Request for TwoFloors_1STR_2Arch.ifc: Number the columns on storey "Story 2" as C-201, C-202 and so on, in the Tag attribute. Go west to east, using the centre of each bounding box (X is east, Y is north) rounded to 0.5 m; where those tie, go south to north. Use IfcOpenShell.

First a look at what the model holds.

```python
import ifcopenshell
import ifcopenshell.util.element
import ifcopenshell.util.placement

model = ifcopenshell.open("TwoFloors_1STR_2Arch.ifc")
print(model.schema)
storey = next(s for s in model.by_type("IfcBuildingStorey") if s.Name == "Story 2")
columns = [e for e in ifcopenshell.util.element.get_decomposition(storey) if e.is_a("IfcColumn")]
for e in sorted(columns, key=lambda e: e.id()):
    origin = ifcopenshell.util.placement.get_local_placement(e.ObjectPlacement)[:3, 3]
    print(e.id(), e.Tag, e.Name, origin.round(2) + 0.0, sep=" | ")
```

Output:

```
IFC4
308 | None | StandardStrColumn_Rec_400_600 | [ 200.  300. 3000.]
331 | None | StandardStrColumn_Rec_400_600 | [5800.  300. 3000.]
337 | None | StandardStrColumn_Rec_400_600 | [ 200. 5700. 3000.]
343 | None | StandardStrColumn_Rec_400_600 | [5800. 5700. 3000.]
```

```python
import ifcopenshell
import ifcopenshell.geom
import ifcopenshell.util.element
import ifcopenshell.util.shape

model = ifcopenshell.open("TwoFloors_1STR_2Arch.ifc")
settings = ifcopenshell.geom.settings()
settings.set("use-world-coords", True)


def centre(element):
    shape = ifcopenshell.geom.create_shape(settings, element)
    return ifcopenshell.util.shape.get_bbox_centroid(shape.geometry)


storey = next(s for s in model.by_type("IfcBuildingStorey") if s.Name == "Story 2")
columns = [e for e in ifcopenshell.util.element.get_decomposition(storey) if e.is_a("IfcColumn")]

# Insertion points can sit at a corner or the storey origin, so sort by the geometry (in metres).
centres = {e: centre(e) for e in columns}
columns.sort(key=lambda e: (round(centres[e][0] / 0.5), centres[e][1]))

for i, e in enumerate(columns, start=1):
    number = f"C-2{i:02d}"
    e.Tag = number
    print(e.id(), number)

model.write("TwoFloors_1STR_2Arch_rev.ifc")
```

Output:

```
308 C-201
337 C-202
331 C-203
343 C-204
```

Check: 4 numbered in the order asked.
